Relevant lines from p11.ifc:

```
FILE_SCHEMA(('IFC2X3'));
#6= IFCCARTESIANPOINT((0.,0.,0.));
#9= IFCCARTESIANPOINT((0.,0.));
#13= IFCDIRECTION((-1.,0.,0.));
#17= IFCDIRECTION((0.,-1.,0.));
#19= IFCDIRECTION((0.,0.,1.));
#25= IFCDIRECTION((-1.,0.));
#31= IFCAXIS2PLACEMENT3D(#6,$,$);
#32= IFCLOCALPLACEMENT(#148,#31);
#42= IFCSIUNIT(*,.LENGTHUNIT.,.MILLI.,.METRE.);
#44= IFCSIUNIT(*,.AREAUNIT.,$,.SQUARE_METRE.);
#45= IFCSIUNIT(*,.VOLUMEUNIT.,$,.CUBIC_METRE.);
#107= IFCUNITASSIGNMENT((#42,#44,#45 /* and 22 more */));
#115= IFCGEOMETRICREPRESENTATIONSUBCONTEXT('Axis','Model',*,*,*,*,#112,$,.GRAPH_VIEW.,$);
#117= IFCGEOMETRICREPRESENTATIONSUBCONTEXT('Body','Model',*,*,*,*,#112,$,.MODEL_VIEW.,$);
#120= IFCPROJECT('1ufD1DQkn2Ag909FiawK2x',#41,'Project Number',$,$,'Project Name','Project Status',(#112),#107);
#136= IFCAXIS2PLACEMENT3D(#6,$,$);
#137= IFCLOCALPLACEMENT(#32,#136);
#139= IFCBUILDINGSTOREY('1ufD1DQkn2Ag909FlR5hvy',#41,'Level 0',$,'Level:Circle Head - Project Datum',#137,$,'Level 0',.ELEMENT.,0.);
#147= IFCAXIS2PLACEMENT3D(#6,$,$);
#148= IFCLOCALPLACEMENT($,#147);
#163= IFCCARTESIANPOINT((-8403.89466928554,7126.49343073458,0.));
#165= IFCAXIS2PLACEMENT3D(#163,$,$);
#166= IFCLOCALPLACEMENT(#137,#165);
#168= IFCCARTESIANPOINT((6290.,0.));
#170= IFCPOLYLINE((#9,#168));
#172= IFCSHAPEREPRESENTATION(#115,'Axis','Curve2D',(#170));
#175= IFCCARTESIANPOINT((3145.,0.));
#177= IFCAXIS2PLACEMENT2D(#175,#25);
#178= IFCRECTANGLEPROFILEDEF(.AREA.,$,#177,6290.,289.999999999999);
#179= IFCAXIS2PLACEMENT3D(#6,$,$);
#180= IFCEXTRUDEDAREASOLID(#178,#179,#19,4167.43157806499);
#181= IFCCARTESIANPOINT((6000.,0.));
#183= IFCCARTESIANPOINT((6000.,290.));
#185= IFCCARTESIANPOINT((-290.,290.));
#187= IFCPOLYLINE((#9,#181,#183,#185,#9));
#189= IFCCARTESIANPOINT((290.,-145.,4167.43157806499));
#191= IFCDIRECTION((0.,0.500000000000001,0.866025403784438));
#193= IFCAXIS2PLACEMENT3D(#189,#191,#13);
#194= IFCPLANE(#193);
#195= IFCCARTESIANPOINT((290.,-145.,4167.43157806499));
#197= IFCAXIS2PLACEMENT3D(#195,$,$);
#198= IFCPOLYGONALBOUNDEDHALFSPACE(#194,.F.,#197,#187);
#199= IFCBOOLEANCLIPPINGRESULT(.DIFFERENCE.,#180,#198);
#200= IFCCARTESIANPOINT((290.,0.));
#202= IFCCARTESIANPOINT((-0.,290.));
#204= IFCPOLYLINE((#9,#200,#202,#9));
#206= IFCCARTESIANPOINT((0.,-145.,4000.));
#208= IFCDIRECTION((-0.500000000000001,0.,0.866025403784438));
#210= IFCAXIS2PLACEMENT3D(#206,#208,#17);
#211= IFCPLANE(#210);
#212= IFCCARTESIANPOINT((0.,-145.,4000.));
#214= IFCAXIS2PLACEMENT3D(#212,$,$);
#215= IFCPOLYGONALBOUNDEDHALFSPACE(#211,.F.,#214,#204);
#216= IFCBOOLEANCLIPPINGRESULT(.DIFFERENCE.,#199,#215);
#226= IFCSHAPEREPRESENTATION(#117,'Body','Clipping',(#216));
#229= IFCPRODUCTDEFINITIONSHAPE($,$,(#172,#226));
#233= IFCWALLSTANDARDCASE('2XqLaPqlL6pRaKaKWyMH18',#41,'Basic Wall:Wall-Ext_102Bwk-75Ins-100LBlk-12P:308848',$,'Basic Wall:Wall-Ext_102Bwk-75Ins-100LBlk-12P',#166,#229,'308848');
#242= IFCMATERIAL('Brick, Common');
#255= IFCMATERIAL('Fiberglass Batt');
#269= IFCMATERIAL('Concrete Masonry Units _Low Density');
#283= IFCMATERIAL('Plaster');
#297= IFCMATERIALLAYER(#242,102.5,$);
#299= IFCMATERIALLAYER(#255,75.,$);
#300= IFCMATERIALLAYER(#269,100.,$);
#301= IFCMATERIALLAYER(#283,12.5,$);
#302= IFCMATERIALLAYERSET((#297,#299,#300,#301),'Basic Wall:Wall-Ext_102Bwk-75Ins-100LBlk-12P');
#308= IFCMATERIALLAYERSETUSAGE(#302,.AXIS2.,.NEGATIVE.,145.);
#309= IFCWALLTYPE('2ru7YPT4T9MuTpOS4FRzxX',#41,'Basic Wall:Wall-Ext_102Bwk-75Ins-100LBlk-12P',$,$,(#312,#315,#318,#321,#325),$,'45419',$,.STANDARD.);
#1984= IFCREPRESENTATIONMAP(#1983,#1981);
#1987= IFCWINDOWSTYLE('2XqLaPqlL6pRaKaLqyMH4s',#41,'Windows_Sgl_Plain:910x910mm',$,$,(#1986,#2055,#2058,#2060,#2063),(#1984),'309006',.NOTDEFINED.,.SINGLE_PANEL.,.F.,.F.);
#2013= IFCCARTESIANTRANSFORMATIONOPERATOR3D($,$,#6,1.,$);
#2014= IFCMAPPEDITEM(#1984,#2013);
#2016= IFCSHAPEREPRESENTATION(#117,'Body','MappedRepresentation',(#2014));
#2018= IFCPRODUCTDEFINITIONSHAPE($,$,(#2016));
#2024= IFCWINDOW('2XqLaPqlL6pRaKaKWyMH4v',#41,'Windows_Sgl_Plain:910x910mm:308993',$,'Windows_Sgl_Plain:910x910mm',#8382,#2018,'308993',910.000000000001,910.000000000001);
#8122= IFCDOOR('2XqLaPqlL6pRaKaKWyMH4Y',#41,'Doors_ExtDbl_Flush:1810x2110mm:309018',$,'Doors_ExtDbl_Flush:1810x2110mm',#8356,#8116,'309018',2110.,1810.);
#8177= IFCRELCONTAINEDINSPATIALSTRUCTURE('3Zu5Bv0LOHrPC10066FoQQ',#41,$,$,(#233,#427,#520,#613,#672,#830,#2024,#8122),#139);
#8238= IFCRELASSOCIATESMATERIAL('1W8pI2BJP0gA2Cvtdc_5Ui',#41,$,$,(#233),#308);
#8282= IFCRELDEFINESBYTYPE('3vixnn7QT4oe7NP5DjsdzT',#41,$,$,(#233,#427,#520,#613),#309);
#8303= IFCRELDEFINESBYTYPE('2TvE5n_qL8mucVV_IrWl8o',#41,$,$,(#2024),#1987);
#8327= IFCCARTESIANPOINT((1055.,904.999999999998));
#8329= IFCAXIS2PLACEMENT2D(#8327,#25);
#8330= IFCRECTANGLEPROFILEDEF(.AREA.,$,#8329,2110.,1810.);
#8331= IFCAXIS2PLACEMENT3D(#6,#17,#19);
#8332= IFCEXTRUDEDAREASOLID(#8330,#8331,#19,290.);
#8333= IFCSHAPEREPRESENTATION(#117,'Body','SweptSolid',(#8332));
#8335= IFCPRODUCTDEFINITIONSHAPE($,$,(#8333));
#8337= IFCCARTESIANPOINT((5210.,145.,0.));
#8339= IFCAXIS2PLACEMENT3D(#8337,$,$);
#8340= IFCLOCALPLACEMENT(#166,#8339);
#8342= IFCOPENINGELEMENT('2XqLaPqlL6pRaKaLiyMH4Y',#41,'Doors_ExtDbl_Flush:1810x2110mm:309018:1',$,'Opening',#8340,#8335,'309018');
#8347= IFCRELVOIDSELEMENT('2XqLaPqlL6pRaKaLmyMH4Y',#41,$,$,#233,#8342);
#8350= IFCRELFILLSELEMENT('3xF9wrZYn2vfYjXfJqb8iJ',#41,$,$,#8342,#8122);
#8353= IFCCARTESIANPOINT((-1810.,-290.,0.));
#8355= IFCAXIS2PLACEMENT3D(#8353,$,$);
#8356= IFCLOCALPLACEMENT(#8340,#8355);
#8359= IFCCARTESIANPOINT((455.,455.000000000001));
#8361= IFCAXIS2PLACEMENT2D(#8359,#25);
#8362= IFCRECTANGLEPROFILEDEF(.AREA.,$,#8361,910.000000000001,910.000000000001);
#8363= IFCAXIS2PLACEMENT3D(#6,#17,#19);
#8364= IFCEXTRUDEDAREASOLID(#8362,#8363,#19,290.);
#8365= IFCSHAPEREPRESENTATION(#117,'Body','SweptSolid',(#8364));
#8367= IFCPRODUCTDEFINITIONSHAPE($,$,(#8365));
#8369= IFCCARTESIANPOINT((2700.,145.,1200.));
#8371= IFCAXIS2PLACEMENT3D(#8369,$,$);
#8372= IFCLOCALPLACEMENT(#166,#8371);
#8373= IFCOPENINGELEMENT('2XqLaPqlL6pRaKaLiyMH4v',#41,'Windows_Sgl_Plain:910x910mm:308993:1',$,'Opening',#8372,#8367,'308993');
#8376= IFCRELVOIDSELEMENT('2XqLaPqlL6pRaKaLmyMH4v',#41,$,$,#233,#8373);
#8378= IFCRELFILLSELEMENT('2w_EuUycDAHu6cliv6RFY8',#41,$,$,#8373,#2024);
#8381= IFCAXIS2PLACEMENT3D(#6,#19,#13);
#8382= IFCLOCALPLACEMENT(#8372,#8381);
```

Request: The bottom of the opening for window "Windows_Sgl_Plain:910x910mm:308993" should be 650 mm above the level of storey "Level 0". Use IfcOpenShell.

```python
import numpy as np
import ifcopenshell
import ifcopenshell.api.geometry
import ifcopenshell.geom
import ifcopenshell.util.element
import ifcopenshell.util.placement
import ifcopenshell.util.shape
import ifcopenshell.util.unit

model = ifcopenshell.open("p11.ifc")
unit_scale = ifcopenshell.util.unit.calculate_unit_scale(model)

window = model.by_guid("2XqLaPqlL6pRaKaKWyMH4v")
opening = window.FillsVoids[0].RelatingOpeningElement
storey = ifcopenshell.util.element.get_container(window, ifc_class="IfcBuildingStorey")
level = ifcopenshell.util.placement.get_local_placement(storey.ObjectPlacement)[2, 3]

# The opening's origin need not be at the sill, so measure its lowest point.
shape = ifcopenshell.geom.create_shape(ifcopenshell.geom.settings(), opening)
bottom = ifcopenshell.util.shape.get_shape_bottom_elevation(shape, shape.geometry) / unit_scale
dz = level + 650.0 - bottom

shift = np.array([0.0, 0.0, dz])
# The window is placed relative to its opening, so it follows when the opening moves.
matrix = ifcopenshell.util.placement.get_local_placement(opening.ObjectPlacement)
matrix[:3, 3] += shift
ifcopenshell.api.geometry.edit_object_placement(
    model, product=opening, matrix=matrix, is_si=False, should_transform_children=True
)

print(f"moved by {dz * unit_scale:+.3f} m")

model.write("p11-out.ifc")
```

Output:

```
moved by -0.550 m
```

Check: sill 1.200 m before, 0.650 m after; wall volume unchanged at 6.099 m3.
